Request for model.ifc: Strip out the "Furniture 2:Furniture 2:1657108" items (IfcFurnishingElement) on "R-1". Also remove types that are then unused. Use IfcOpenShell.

First a look at what the model holds.

```python
import ifcopenshell
import ifcopenshell.util.element

model = ifcopenshell.open("model.ifc")
print(model.schema)
storey = next(s for s in model.by_type("IfcBuildingStorey") if s.Name == "R-1")
furniture = [e for e in ifcopenshell.util.element.get_decomposition(storey) if e.is_a("IfcFurnishingElement")]
seen = {}
for e in furniture:
    element_type = ifcopenshell.util.element.get_type(e)
    name = element_type.Name if element_type not in (None, e) else None
    seen[name] = seen.get(name, 0) + 1
for name, count in sorted(seen.items(), key=str):
    print(count, "x", name)
```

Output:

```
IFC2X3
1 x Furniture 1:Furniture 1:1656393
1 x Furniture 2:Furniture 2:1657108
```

```python
import ifcopenshell
import ifcopenshell.api.root
import ifcopenshell.util.element

model = ifcopenshell.open("model.ifc")

storey = next(s for s in model.by_type("IfcBuildingStorey") if s.Name == "R-1")
furniture = [e for e in ifcopenshell.util.element.get_decomposition(storey) if e.is_a("IfcFurnishingElement")]
targets = [e for e in furniture if (t := ifcopenshell.util.element.get_type(e)) not in (None, e) and t.Name == "Furniture 2:Furniture 2:1657108"]
types = {ifcopenshell.util.element.get_type(e) for e in targets} - {None, *targets}

for e in targets:
    ifcopenshell.api.root.remove_product(model, product=e)
print(len(targets), "removed")

unused = [t for t in types if not ifcopenshell.util.element.get_types(t)]
for t in unused:
    ifcopenshell.api.root.remove_product(model, product=t)
print(len(unused), "unused types removed")

model.write("model_v2.ifc")
```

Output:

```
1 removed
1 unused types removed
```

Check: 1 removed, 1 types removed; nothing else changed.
